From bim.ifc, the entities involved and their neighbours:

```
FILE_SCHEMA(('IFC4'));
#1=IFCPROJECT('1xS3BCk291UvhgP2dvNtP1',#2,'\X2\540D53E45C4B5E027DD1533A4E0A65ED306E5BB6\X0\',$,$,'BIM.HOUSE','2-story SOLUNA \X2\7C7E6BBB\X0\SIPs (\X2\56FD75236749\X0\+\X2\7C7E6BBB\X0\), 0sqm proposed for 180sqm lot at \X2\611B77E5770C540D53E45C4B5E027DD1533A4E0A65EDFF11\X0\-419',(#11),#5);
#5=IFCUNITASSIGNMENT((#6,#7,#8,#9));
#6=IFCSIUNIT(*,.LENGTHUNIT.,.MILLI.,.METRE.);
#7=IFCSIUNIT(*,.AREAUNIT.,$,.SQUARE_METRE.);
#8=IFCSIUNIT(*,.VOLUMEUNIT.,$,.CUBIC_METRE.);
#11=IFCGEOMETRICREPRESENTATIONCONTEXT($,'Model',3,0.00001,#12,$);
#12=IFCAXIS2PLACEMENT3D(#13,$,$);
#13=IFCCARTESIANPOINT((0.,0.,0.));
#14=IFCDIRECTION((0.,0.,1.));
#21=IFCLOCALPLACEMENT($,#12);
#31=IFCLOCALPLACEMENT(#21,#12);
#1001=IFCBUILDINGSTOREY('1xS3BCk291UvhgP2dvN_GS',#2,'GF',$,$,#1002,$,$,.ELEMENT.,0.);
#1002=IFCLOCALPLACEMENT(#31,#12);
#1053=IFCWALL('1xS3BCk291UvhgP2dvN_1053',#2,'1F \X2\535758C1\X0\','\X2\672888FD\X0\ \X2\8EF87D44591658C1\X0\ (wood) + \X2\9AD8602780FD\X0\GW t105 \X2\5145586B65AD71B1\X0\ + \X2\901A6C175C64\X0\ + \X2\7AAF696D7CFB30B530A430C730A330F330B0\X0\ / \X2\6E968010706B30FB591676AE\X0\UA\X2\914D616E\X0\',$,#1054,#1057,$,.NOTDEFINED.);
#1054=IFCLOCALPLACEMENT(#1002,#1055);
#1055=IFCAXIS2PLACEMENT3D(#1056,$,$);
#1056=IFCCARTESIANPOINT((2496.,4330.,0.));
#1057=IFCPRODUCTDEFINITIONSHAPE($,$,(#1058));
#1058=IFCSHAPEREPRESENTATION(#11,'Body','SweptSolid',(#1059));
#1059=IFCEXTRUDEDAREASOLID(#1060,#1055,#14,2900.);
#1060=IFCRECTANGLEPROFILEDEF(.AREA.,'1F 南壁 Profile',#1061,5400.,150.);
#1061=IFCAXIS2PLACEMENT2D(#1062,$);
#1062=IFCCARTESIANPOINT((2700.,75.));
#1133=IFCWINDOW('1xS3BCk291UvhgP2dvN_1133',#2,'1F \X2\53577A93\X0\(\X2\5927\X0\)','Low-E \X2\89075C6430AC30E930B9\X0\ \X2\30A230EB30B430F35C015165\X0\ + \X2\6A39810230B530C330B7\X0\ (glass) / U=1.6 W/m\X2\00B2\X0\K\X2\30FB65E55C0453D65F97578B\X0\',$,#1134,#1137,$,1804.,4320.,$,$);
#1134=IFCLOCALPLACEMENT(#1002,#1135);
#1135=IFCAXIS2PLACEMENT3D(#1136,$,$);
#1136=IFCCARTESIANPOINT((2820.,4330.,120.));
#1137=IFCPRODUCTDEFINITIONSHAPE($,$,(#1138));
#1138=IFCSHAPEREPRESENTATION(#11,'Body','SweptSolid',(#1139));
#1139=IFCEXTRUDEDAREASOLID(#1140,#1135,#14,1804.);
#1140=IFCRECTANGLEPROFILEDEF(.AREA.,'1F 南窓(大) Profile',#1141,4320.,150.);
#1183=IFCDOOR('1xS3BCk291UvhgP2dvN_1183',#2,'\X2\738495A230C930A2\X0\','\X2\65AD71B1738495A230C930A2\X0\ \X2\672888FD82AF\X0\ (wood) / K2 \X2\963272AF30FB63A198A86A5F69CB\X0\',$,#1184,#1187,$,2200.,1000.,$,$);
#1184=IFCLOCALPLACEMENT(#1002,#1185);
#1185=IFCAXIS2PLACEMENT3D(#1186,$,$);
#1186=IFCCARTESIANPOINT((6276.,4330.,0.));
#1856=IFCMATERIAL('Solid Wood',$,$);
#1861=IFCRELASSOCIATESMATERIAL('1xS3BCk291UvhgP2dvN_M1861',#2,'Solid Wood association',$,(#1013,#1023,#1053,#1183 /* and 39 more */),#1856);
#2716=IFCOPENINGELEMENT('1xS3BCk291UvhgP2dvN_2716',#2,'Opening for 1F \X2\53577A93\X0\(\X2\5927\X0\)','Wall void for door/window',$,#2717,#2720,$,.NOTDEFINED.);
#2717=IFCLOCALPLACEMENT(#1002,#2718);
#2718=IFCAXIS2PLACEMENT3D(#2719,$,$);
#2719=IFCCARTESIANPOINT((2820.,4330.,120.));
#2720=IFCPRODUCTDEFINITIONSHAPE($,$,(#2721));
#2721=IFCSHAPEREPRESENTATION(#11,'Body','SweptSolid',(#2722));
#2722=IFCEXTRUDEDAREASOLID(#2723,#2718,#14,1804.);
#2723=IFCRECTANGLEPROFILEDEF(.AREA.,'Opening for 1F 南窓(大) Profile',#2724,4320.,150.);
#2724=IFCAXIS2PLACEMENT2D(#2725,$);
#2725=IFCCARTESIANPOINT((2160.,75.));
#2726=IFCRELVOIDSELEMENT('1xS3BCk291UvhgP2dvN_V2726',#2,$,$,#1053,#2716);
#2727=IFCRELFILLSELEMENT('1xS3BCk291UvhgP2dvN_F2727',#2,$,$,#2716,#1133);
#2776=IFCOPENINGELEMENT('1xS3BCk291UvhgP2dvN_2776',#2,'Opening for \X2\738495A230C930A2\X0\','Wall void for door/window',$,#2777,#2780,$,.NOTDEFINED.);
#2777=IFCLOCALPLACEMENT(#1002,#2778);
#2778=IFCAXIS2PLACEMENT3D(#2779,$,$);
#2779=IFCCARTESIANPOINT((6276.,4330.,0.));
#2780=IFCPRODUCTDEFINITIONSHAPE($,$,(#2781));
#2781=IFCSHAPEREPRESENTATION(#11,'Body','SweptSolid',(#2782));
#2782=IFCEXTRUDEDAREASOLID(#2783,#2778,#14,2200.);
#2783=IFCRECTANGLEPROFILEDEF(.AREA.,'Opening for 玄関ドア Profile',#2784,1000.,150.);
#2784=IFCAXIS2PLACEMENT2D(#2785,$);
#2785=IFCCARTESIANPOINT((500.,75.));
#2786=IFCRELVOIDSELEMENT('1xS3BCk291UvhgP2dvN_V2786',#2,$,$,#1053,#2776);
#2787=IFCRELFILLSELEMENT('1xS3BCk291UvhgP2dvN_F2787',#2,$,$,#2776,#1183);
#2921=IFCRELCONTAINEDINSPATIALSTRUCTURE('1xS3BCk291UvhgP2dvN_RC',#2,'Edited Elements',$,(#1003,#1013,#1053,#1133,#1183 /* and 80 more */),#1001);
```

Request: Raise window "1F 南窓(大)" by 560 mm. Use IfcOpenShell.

```python
import numpy as np
import ifcopenshell
import ifcopenshell.api.geometry
import ifcopenshell.util.placement
import ifcopenshell.util.unit

model = ifcopenshell.open("bim.ifc")
unit_scale = ifcopenshell.util.unit.calculate_unit_scale(model)

window = model.by_guid("1xS3BCk291UvhgP2dvN_1133")
opening = window.FillsVoids[0].RelatingOpeningElement
dz = 0.56 / unit_scale

shift = np.array([0.0, 0.0, dz])
# The window is not placed relative to its opening, so move both.
for product in (opening, window):
    matrix = ifcopenshell.util.placement.get_local_placement(product.ObjectPlacement)
    matrix[:3, 3] += shift
    ifcopenshell.api.geometry.edit_object_placement(model, product=product, matrix=matrix, is_si=False)

print(f"moved by {dz * unit_scale:+.3f} m")

model.write("bim_v2.ifc")
```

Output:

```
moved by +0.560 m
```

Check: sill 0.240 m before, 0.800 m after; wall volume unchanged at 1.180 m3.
